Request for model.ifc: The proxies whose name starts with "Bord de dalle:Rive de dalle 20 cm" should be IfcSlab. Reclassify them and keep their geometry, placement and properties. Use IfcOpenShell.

First a look at what the model holds.

```python
import re

import ifcopenshell

model = ifcopenshell.open("model.ifc")
print(model.schema)
seen = {}
for e in model.by_type("IfcBuildingElementProxy"):
    name = re.sub(r":\d+(:\d+)?$", "", e.Name or "")  # drop the element id that some exporters append
    seen[name] = seen.get(name, 0) + 1
for name, count in sorted(seen.items()):
    print(count, "x", name)
```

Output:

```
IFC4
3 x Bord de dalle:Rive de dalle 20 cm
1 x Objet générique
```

```python
import ifcopenshell
import ifcopenshell.api.root

model = ifcopenshell.open("model.ifc")

proxies = [e.id() for e in model.by_type("IfcBuildingElementProxy") if (e.Name or "").startswith("Bord de dalle:Rive de dalle 20 cm")]
for step_id in proxies:
    proxy = model.by_id(step_id)
    # Reclassifying a typed element also reclassifies its type and the type's other occurrences.
    if proxy.is_a("IfcBuildingElementProxy"):
        ifcopenshell.api.root.reassign_class(model, product=proxy, ifc_class="IfcSlab", predefined_type="FLOOR")

print(sum(model.by_id(i).is_a("IfcSlab") for i in proxies), "reclassified")

model.write("model_v2.ifc")
```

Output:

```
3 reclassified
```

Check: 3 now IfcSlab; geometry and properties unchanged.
